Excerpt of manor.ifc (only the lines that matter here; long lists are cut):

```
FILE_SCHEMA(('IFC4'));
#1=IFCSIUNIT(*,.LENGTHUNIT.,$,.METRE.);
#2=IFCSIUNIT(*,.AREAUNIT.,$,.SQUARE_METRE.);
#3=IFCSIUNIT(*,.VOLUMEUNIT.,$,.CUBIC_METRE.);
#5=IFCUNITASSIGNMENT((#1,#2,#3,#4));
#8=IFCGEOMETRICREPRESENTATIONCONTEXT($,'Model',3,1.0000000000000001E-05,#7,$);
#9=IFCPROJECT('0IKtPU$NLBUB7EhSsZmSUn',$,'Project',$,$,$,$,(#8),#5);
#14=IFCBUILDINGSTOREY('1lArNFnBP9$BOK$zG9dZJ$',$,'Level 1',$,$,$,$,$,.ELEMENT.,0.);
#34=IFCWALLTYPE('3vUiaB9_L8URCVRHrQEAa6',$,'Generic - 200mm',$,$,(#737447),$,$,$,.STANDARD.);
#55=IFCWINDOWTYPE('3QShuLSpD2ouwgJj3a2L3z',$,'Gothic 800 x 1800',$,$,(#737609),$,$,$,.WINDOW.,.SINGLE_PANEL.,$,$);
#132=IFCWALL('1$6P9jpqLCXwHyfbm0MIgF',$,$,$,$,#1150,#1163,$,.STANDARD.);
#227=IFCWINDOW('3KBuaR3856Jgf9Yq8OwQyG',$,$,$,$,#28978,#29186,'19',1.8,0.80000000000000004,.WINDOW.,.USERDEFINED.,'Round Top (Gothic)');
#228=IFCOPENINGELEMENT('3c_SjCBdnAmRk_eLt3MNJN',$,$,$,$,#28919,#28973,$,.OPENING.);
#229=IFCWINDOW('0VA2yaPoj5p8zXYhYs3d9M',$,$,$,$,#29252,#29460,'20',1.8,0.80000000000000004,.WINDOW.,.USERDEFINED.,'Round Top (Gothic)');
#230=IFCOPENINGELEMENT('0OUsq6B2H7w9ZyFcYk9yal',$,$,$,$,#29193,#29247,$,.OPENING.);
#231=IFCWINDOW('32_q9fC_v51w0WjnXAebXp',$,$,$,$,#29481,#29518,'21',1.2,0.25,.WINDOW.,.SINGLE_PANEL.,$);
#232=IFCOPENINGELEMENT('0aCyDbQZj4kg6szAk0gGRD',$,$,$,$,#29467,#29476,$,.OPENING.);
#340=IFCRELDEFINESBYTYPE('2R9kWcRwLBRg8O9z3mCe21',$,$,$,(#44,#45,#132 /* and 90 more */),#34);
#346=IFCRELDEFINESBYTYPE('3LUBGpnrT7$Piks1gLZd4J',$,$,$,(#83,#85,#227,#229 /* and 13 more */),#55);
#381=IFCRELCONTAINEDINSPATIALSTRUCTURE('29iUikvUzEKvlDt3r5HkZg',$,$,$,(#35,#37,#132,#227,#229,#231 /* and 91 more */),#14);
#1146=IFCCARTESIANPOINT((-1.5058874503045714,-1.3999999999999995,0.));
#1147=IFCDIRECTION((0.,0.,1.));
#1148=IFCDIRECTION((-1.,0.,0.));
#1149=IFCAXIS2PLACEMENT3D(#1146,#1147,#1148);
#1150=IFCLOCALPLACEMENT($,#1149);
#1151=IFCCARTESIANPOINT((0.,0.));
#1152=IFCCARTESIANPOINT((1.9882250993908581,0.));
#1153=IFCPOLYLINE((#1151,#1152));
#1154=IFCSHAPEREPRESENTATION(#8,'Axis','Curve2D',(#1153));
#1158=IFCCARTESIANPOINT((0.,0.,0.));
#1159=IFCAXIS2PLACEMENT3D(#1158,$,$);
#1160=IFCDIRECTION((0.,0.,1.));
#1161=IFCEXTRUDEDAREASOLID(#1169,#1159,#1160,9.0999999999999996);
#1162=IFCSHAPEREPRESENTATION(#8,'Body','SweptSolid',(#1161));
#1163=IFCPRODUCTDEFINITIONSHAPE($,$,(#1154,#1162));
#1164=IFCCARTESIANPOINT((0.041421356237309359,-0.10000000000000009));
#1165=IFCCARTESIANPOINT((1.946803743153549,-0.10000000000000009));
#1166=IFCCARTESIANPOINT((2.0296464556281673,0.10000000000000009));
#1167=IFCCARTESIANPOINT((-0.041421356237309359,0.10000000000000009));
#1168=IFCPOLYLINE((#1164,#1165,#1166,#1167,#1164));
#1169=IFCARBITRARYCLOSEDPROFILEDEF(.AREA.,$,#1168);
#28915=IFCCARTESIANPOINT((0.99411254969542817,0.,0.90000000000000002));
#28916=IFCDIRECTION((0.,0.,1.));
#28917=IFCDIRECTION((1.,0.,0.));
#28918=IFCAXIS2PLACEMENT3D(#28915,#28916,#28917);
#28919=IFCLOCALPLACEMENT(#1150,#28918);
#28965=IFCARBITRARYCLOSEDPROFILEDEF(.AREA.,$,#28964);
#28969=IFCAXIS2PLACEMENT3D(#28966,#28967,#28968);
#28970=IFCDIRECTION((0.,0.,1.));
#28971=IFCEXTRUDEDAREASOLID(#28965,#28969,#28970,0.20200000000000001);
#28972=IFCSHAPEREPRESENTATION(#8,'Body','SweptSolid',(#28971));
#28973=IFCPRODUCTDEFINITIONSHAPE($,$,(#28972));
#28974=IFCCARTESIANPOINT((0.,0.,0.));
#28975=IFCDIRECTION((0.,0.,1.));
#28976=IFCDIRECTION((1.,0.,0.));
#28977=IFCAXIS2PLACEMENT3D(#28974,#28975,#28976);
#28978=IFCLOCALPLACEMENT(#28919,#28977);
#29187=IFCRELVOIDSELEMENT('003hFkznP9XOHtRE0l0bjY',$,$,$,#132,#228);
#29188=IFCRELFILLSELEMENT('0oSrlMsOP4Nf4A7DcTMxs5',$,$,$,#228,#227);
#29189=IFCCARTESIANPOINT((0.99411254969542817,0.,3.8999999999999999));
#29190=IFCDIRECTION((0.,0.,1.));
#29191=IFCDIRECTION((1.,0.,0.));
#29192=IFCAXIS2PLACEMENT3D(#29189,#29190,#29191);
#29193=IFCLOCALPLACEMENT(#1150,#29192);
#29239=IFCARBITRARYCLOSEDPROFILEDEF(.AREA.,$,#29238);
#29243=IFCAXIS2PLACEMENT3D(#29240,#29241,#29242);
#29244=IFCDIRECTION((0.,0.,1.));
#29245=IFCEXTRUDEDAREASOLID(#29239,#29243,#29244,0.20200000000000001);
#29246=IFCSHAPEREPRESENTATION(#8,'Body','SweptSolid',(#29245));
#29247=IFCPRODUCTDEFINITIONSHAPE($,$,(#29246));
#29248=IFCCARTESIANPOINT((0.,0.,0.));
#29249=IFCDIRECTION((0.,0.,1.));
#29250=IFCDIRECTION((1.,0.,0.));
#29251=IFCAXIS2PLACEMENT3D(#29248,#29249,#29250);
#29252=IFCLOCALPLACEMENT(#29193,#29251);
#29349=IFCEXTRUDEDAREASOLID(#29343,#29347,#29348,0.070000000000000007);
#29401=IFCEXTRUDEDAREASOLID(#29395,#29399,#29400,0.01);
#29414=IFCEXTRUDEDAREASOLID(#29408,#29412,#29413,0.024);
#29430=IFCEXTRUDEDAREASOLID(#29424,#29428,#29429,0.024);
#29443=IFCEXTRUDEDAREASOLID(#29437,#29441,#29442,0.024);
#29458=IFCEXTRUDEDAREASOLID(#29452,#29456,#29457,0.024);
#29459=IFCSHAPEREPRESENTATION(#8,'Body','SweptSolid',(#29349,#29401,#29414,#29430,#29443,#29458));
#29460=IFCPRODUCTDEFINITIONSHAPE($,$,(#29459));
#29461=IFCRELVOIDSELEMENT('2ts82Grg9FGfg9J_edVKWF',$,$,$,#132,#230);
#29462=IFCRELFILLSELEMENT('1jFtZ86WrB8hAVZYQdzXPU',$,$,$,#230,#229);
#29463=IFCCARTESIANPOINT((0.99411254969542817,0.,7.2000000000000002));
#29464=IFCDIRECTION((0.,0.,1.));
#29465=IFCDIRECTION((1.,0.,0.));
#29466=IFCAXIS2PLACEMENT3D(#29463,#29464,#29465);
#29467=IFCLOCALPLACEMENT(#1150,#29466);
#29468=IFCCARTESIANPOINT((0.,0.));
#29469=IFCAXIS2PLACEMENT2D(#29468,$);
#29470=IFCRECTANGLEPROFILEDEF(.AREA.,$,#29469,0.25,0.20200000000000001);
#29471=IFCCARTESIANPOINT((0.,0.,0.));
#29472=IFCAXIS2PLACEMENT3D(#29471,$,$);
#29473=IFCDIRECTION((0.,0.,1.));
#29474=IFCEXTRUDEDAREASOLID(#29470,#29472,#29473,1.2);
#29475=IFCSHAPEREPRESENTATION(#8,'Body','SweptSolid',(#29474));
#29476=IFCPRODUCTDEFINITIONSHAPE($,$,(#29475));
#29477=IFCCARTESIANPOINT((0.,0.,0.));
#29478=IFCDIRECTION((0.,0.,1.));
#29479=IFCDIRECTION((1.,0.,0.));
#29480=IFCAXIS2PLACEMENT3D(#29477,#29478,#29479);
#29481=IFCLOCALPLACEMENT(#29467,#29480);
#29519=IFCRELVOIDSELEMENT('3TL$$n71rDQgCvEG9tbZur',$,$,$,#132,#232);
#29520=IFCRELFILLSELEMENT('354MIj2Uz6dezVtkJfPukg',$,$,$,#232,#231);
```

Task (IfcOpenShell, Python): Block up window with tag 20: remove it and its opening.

```python
import ifcopenshell
import ifcopenshell.api.feature
import ifcopenshell.api.root
import ifcopenshell.geom
import ifcopenshell.util.shape

model = ifcopenshell.open("manor.ifc")
settings = ifcopenshell.geom.settings()


def volume(element):
    """Net volume in cubic metres, openings subtracted."""
    shape = ifcopenshell.geom.create_shape(settings, element)
    return ifcopenshell.util.shape.get_volume(shape.geometry)


window = model.by_id(229)
opening = window.FillsVoids[0].RelatingOpeningElement
wall = opening.VoidsElements[0].RelatingBuildingElement
before = volume(wall)

ifcopenshell.api.root.remove_product(model, product=window)
ifcopenshell.api.feature.remove_feature(model, feature=opening)

after = volume(wall)

print(f"wall volume {before:.3f} -> {after:.3f} m3")

model.write("manor_v2.ifc")
```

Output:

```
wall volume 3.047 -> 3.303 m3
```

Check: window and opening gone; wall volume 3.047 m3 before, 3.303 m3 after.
